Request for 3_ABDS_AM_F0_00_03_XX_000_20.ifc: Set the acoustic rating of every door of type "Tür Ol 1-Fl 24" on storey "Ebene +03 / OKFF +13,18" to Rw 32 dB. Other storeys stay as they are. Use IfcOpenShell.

First a look at what the model holds.

```python
import ifcopenshell
import ifcopenshell.util.element

model = ifcopenshell.open("3_ABDS_AM_F0_00_03_XX_000_20.ifc")
print(model.schema)
storey = next(s for s in model.by_type("IfcBuildingStorey") if s.Name == "Ebene +03 / OKFF +13,18")
doors = [e for e in ifcopenshell.util.element.get_decomposition(storey) if e.is_a("IfcDoor")]
seen = {}
for e in doors:
    element_type = ifcopenshell.util.element.get_type(e)
    key = (element_type.Name if element_type != e and element_type else None, ifcopenshell.util.element.get_pset(e, "Pset_DoorCommon", "AcousticRating"))
    seen[key] = seen.get(key, 0) + 1
for (name, value), count in sorted(seen.items(), key=str):
    print(count, "x", name, "|", value)
```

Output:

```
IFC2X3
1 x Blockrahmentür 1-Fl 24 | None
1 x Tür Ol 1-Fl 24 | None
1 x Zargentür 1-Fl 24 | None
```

```python
import ifcopenshell
import ifcopenshell.api.pset
import ifcopenshell.util.element

model = ifcopenshell.open("3_ABDS_AM_F0_00_03_XX_000_20.ifc")

storey = next(s for s in model.by_type("IfcBuildingStorey") if s.Name == "Ebene +03 / OKFF +13,18")
doors = [e for e in ifcopenshell.util.element.get_decomposition(storey) if e.is_a("IfcDoor")]

count = 0
for e in doors:
    element_type = ifcopenshell.util.element.get_type(e)
    if element_type in (None, e) or element_type.Name != "Tür Ol 1-Fl 24":
        continue
    # add_pset returns the element's existing set when there is one.
    pset = ifcopenshell.api.pset.add_pset(model, product=e, name="Pset_DoorCommon")
    ifcopenshell.api.pset.edit_pset(model, pset=pset, properties={"AcousticRating": "Rw 32 dB"})
    count += 1

print(count, "doors updated")

model.write("3_ABDS_AM_F0_00_03_XX_000_20_v2.ifc")
```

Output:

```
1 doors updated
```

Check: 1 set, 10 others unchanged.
